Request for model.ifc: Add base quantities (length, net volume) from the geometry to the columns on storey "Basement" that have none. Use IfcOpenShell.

First a look at what the model holds.

```python
import ifcopenshell
import ifcopenshell.util.element
import ifcopenshell.util.unit

model = ifcopenshell.open("model.ifc")
print(model.schema)
for unit_type in ("LENGTHUNIT", "AREAUNIT", "VOLUMEUNIT"):
    print(unit_type, ifcopenshell.util.unit.calculate_unit_scale(model, unit_type))
storey = next(s for s in model.by_type("IfcBuildingStorey") if s.Name == "Basement")
columns = [e for e in ifcopenshell.util.element.get_decomposition(storey) if e.is_a("IfcColumn")]
for e in sorted(columns, key=lambda e: e.id()):
    print(e.id(), e.is_a(), e.Name, list(ifcopenshell.util.element.get_psets(e, qtos_only=True)), sep=" | ")
```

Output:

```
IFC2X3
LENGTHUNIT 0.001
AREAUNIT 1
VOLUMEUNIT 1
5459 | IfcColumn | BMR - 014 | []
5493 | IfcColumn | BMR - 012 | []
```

```python
import ifcopenshell
import ifcopenshell.api.pset
import ifcopenshell.geom
import ifcopenshell.util.element
import ifcopenshell.util.shape
import ifcopenshell.util.unit

model = ifcopenshell.open("model.ifc")
unit_scale = ifcopenshell.util.unit.calculate_unit_scale(model)
volume_scale = ifcopenshell.util.unit.calculate_unit_scale(model, "VOLUMEUNIT")
settings = ifcopenshell.geom.settings()

storey = next(s for s in model.by_type("IfcBuildingStorey") if s.Name == "Basement")
columns = [e for e in ifcopenshell.util.element.get_decomposition(storey) if e.is_a("IfcColumn")]

for e in sorted(columns, key=lambda e: e.id()):
    if ifcopenshell.util.element.get_psets(e, qtos_only=True, should_inherit=False):
        continue
    # Geometry comes back in metres, in the element's own axes.
    shape = ifcopenshell.geom.create_shape(settings, e)
    values = {
        "Length": ifcopenshell.util.shape.get_z(shape.geometry) / unit_scale,
        "NetVolume": ifcopenshell.util.shape.get_volume(shape.geometry) / volume_scale,
    }
    qto = ifcopenshell.api.pset.add_qto(model, product=e, name="BaseQuantities")
    ifcopenshell.api.pset.edit_qto(model, qto=qto, properties=values)
    print(e.id(), {k: round(v, 3) for k, v in values.items()})

model.write("model_updated.ifc")
```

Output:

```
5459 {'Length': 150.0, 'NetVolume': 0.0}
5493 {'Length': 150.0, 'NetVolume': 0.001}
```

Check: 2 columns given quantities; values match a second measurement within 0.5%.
